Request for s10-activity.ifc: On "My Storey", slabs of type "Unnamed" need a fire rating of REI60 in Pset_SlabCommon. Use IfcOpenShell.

First a look at what the model holds.

```python
import ifcopenshell
import ifcopenshell.util.element

model = ifcopenshell.open("s10-activity.ifc")
print(model.schema)
storey = next(s for s in model.by_type("IfcBuildingStorey") if s.Name == "My Storey")
slabs = [e for e in ifcopenshell.util.element.get_decomposition(storey) if e.is_a("IfcSlab")]
seen = {}
for e in slabs:
    element_type = ifcopenshell.util.element.get_type(e)
    key = (element_type.Name if element_type != e and element_type else None, ifcopenshell.util.element.get_pset(e, "Pset_SlabCommon", "FireRating"))
    seen[key] = seen.get(key, 0) + 1
for (name, value), count in sorted(seen.items(), key=str):
    print(count, "x", name, "|", value)
```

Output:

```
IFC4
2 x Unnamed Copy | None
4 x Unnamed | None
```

```python
import ifcopenshell
import ifcopenshell.api.pset
import ifcopenshell.util.element

model = ifcopenshell.open("s10-activity.ifc")

storey = next(s for s in model.by_type("IfcBuildingStorey") if s.Name == "My Storey")
slabs = [e for e in ifcopenshell.util.element.get_decomposition(storey) if e.is_a("IfcSlab")]

count = 0
for e in slabs:
    element_type = ifcopenshell.util.element.get_type(e)
    if element_type in (None, e) or element_type.Name != "Unnamed":
        continue
    # add_pset returns the element's existing set when there is one.
    pset = ifcopenshell.api.pset.add_pset(model, product=e, name="Pset_SlabCommon")
    ifcopenshell.api.pset.edit_pset(model, pset=pset, properties={"FireRating": "REI60"})
    count += 1

print(count, "slabs updated")

model.write("s10-activity_v2.ifc")
```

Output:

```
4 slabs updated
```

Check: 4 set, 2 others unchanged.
